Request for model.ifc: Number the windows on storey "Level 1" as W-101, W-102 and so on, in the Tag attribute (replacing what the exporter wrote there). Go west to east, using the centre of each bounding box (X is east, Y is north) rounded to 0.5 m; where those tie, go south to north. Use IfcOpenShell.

First a look at what the model holds.

```python
import ifcopenshell
import ifcopenshell.util.element
import ifcopenshell.util.placement

model = ifcopenshell.open("model.ifc")
print(model.schema)
storey = next(s for s in model.by_type("IfcBuildingStorey") if s.Name == "Level 1")
windows = [e for e in ifcopenshell.util.element.get_decomposition(storey) if e.is_a("IfcWindow")]
for e in sorted(windows, key=lambda e: e.id()):
    origin = ifcopenshell.util.placement.get_local_placement(e.ObjectPlacement)[:3, 3]
    print(e.id(), e.Tag, e.Name, origin.round(2) + 0.0, sep=" | ")
```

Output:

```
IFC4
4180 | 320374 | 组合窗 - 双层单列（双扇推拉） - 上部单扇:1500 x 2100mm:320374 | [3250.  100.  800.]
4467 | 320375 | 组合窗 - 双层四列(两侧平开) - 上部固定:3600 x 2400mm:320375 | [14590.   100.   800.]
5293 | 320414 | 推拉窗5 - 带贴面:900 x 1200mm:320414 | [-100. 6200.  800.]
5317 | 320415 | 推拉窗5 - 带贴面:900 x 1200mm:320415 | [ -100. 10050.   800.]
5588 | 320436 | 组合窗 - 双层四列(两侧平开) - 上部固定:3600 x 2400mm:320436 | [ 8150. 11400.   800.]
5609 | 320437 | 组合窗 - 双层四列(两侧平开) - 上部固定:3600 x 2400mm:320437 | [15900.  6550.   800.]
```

```python
import ifcopenshell
import ifcopenshell.geom
import ifcopenshell.util.element
import ifcopenshell.util.shape

model = ifcopenshell.open("model.ifc")
settings = ifcopenshell.geom.settings()
settings.set("use-world-coords", True)


def centre(element):
    shape = ifcopenshell.geom.create_shape(settings, element)
    return ifcopenshell.util.shape.get_bbox_centroid(shape.geometry)


storey = next(s for s in model.by_type("IfcBuildingStorey") if s.Name == "Level 1")
windows = [e for e in ifcopenshell.util.element.get_decomposition(storey) if e.is_a("IfcWindow")]

# Insertion points can sit at a corner or the storey origin, so sort by the geometry (in metres).
centres = {e: centre(e) for e in windows}
windows.sort(key=lambda e: (round(centres[e][0] / 0.5), centres[e][1]))

for i, e in enumerate(windows, start=1):
    number = f"W-1{i:02d}"
    e.Tag = number
    print(e.id(), number)

model.write("model_edited.ifc")
```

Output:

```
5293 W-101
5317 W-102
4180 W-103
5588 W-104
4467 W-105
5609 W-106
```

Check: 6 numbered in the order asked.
